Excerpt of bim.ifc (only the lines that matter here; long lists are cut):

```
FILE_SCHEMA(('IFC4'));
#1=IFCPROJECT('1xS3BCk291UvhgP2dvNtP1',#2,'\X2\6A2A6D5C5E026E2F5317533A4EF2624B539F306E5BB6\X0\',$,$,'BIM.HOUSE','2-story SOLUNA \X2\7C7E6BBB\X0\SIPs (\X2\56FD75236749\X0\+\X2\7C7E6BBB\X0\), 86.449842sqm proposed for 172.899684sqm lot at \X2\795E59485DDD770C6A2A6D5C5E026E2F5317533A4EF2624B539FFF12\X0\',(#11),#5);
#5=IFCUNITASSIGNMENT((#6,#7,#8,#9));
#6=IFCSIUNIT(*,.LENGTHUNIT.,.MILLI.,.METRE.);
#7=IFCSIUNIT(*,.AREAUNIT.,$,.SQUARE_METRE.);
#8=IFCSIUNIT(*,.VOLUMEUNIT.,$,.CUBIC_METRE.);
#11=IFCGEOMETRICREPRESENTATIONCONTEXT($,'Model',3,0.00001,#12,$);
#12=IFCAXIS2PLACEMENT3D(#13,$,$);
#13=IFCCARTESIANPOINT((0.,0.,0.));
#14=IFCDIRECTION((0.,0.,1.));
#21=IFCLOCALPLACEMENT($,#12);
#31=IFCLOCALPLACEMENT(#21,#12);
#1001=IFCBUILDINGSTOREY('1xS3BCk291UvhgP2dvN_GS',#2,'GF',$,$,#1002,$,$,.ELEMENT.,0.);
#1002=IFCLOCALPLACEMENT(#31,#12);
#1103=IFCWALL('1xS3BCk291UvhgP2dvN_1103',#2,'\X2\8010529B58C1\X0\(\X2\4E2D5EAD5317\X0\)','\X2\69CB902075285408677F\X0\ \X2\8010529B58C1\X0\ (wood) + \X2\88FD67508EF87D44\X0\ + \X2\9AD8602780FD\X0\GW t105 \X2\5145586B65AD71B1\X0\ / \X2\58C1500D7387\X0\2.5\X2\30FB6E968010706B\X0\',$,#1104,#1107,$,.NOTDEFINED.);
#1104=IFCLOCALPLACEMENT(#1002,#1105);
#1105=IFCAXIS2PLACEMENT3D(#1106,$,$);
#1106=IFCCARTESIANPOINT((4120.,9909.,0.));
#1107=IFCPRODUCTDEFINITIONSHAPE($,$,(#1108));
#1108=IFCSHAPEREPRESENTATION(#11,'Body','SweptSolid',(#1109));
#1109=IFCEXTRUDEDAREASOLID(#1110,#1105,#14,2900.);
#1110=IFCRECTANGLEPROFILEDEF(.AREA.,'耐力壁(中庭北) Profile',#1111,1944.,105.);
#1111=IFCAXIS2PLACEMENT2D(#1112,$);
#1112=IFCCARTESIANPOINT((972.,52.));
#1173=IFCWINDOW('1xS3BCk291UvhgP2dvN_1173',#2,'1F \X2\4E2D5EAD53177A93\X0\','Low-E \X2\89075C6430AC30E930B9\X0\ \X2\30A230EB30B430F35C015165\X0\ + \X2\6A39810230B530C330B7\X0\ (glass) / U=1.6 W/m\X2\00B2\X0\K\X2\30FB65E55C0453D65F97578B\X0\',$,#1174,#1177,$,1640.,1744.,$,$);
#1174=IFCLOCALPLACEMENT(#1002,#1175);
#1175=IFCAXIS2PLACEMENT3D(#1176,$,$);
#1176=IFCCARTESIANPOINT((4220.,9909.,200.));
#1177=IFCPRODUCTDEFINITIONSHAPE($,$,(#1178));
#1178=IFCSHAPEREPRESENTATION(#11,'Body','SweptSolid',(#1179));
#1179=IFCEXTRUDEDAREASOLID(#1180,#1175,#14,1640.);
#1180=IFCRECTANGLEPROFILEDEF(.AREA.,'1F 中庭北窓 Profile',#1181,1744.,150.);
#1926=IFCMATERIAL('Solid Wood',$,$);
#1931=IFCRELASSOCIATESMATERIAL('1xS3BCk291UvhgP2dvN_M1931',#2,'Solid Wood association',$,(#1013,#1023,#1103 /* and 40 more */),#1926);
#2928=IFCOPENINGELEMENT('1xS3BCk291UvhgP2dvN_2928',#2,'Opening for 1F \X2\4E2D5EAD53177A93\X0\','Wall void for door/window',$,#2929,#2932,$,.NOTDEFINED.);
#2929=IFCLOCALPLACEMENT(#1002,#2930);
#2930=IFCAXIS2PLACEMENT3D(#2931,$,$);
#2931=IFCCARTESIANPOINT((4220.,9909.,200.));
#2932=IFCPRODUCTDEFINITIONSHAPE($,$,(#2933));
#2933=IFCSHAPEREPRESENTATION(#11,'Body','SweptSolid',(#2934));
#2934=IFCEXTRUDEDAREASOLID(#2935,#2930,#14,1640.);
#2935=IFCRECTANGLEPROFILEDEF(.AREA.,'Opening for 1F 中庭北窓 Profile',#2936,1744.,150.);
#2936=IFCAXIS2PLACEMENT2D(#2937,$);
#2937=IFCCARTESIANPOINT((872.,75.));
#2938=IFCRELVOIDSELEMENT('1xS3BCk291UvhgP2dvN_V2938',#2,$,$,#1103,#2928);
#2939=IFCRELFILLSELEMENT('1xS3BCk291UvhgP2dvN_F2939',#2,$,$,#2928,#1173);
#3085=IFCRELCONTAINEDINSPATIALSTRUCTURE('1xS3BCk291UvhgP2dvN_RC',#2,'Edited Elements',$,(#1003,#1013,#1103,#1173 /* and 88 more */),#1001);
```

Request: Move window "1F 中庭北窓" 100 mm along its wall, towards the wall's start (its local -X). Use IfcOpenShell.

```python
import ifcopenshell
import ifcopenshell.api.geometry
import ifcopenshell.util.placement
import ifcopenshell.util.unit

model = ifcopenshell.open("bim.ifc")
unit_scale = ifcopenshell.util.unit.calculate_unit_scale(model)

window = model.by_id(1173)
opening = window.FillsVoids[0].RelatingOpeningElement
wall = opening.VoidsElements[0].RelatingBuildingElement

wall_matrix = ifcopenshell.util.placement.get_local_placement(wall.ObjectPlacement)
shift = wall_matrix[:3, 0] * -0.1 / unit_scale
before = ifcopenshell.util.placement.get_local_placement(window.ObjectPlacement)[:3, 3].copy()

# The window is not placed relative to its opening, so move both.
for product in (opening, window):
    matrix = ifcopenshell.util.placement.get_local_placement(product.ObjectPlacement)
    matrix[:3, 3] += shift
    ifcopenshell.api.geometry.edit_object_placement(model, product=product, matrix=matrix, is_si=False)

after = ifcopenshell.util.placement.get_local_placement(window.ObjectPlacement)[:3, 3]
print("window moved by", (after - before).round(3) + 0.0)

model.write("bim-out.ifc")
```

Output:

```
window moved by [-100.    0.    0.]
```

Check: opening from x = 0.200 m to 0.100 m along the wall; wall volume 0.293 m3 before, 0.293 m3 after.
